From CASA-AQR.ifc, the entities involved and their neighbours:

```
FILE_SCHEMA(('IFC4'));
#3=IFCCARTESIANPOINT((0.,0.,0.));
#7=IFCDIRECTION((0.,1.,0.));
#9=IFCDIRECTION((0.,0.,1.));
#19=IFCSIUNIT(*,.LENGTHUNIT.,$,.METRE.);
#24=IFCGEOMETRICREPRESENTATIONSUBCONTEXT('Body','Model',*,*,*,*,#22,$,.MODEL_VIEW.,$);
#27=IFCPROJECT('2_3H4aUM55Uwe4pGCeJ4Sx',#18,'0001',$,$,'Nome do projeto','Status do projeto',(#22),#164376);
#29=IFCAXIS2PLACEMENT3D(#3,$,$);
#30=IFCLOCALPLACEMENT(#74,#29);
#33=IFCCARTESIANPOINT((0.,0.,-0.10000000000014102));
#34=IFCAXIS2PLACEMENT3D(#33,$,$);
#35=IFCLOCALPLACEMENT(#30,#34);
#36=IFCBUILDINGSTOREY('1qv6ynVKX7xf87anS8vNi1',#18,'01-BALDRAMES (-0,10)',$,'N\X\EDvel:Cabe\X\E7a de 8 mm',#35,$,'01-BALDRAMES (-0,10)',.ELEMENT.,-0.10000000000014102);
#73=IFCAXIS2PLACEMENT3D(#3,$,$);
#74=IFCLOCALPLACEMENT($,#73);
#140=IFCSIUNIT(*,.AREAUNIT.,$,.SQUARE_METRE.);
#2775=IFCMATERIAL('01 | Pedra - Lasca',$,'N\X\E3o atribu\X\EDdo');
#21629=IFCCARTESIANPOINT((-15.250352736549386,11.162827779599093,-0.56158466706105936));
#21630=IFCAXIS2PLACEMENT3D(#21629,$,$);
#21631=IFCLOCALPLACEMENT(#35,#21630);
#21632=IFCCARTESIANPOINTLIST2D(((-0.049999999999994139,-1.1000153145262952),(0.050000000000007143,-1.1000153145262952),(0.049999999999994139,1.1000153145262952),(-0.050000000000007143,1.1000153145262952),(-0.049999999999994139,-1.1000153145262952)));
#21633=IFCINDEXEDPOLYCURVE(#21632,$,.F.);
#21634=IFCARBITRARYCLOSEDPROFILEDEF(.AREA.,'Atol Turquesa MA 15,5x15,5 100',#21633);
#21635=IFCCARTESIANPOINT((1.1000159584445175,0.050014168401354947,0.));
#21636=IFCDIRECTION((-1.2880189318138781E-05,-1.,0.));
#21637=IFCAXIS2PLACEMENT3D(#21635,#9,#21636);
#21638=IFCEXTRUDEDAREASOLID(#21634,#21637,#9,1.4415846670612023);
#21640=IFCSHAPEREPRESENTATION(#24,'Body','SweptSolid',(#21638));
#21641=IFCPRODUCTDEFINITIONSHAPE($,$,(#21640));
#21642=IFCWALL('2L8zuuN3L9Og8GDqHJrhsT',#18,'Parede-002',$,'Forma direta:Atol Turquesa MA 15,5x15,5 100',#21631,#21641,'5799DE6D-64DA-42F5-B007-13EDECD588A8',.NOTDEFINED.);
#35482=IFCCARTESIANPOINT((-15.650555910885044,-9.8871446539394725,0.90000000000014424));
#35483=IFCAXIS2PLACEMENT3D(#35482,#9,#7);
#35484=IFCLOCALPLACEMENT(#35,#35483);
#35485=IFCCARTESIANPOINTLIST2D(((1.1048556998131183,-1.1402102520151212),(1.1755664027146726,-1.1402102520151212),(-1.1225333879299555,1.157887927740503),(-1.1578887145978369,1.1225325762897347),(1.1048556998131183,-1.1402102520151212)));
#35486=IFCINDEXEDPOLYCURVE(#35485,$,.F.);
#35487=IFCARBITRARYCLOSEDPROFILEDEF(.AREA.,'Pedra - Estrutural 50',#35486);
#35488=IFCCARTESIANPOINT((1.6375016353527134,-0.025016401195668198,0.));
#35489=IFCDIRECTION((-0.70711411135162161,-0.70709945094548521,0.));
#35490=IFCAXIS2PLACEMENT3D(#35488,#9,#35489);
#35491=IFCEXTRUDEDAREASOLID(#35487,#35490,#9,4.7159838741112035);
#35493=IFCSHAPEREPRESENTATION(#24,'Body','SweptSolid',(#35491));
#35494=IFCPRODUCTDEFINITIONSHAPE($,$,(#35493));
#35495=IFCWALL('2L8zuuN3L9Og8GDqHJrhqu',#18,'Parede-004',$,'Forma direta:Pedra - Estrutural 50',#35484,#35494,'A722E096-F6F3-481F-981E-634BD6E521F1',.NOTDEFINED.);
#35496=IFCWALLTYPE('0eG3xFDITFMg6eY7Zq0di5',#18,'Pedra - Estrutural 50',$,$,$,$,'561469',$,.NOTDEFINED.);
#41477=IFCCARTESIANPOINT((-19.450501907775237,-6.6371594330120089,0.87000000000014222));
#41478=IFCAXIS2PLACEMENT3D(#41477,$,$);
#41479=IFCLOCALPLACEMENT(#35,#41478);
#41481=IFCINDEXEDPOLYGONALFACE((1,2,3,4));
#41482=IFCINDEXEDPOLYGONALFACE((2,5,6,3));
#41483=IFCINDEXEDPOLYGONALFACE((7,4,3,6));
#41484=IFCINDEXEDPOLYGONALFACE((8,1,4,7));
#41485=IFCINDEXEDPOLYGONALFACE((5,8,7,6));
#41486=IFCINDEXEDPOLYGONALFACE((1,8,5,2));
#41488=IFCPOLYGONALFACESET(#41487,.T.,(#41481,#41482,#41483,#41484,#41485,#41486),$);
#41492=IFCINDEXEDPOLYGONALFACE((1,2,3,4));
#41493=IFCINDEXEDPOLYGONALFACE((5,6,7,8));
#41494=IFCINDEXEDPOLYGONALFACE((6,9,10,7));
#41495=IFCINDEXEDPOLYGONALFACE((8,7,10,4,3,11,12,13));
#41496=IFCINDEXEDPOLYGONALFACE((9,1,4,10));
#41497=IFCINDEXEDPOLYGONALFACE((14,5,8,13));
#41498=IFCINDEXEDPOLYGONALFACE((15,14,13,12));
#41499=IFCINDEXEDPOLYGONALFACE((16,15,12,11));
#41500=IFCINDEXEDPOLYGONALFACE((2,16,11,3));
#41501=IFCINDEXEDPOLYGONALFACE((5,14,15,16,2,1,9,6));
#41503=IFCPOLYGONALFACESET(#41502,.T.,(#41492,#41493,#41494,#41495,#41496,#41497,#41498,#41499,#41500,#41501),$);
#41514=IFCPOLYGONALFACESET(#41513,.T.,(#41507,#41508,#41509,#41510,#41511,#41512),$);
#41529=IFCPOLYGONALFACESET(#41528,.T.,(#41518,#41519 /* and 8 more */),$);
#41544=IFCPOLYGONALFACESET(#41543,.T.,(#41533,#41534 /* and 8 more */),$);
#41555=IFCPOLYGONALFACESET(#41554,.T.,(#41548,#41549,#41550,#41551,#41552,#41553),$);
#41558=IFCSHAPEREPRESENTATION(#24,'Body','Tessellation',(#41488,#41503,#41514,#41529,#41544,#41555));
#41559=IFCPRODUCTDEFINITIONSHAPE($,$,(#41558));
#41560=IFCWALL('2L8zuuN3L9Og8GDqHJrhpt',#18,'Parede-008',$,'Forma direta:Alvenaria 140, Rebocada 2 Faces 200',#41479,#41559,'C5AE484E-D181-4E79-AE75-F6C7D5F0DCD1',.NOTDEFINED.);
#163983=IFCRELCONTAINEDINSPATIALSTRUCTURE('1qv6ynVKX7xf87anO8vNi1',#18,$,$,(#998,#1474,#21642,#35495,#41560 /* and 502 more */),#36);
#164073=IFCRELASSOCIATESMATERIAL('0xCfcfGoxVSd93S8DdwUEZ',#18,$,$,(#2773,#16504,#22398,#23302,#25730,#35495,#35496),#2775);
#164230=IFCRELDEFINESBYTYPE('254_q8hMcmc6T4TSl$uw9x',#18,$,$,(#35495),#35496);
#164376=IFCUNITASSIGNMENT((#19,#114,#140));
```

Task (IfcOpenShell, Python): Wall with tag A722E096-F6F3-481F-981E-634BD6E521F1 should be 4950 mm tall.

```python
import ifcopenshell
import ifcopenshell.geom
import ifcopenshell.util.representation
import ifcopenshell.util.shape
import ifcopenshell.util.unit

model = ifcopenshell.open("CASA-AQR.ifc")
unit_scale = ifcopenshell.util.unit.calculate_unit_scale(model)
settings = ifcopenshell.geom.settings()


def volume(element):
    """Net volume in cubic metres, openings subtracted."""
    shape = ifcopenshell.geom.create_shape(settings, element)
    return ifcopenshell.util.shape.get_volume(shape.geometry)


wall = model.by_guid("2L8zuuN3L9Og8GDqHJrhqu")
before = volume(wall)

body = ifcopenshell.util.representation.get_representation(wall, "Model", "Body")
solid = body.Items[0]
old_height = solid.Depth
solid.Depth = 4.95 / unit_scale
after = volume(wall)

print(f"height {old_height:g} -> {solid.Depth:g}, volume {before:.3f} -> {after:.3f} m3")

model.write("CASA-AQR_rev.ifc")
```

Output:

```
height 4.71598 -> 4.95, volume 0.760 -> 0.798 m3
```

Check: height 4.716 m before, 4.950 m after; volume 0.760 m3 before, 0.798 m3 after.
